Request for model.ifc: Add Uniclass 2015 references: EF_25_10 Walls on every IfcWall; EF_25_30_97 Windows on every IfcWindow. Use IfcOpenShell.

First a look at what the model holds.

```python
import ifcopenshell

model = ifcopenshell.open("model.ifc")
print(model.schema)
print("classifications:", [c.Name for c in model.by_type("IfcClassification")])
for ifc_class in ("IfcDoor", "IfcRoof", "IfcStair", "IfcWall", "IfcWindow"):
    print(ifc_class, len(model.by_type(ifc_class)))
```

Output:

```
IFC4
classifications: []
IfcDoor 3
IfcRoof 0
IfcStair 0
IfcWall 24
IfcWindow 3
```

```python
import ifcopenshell
import ifcopenshell.api.classification

model = ifcopenshell.open("model.ifc")

system = ifcopenshell.api.classification.add_classification(model, classification="Uniclass 2015")

codes = {
    "IfcWall": ("EF_25_10", "Walls"),
    "IfcWindow": ("EF_25_30_97", "Windows"),
}
for ifc_class, (code, name) in codes.items():
    products = model.by_type(ifc_class)
    ifcopenshell.api.classification.add_reference(
        model, products=products, classification=system, identification=code, name=name
    )
    print(code, len(products))

model.write("model_rev.ifc")
```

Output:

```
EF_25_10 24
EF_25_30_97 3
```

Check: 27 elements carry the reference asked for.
